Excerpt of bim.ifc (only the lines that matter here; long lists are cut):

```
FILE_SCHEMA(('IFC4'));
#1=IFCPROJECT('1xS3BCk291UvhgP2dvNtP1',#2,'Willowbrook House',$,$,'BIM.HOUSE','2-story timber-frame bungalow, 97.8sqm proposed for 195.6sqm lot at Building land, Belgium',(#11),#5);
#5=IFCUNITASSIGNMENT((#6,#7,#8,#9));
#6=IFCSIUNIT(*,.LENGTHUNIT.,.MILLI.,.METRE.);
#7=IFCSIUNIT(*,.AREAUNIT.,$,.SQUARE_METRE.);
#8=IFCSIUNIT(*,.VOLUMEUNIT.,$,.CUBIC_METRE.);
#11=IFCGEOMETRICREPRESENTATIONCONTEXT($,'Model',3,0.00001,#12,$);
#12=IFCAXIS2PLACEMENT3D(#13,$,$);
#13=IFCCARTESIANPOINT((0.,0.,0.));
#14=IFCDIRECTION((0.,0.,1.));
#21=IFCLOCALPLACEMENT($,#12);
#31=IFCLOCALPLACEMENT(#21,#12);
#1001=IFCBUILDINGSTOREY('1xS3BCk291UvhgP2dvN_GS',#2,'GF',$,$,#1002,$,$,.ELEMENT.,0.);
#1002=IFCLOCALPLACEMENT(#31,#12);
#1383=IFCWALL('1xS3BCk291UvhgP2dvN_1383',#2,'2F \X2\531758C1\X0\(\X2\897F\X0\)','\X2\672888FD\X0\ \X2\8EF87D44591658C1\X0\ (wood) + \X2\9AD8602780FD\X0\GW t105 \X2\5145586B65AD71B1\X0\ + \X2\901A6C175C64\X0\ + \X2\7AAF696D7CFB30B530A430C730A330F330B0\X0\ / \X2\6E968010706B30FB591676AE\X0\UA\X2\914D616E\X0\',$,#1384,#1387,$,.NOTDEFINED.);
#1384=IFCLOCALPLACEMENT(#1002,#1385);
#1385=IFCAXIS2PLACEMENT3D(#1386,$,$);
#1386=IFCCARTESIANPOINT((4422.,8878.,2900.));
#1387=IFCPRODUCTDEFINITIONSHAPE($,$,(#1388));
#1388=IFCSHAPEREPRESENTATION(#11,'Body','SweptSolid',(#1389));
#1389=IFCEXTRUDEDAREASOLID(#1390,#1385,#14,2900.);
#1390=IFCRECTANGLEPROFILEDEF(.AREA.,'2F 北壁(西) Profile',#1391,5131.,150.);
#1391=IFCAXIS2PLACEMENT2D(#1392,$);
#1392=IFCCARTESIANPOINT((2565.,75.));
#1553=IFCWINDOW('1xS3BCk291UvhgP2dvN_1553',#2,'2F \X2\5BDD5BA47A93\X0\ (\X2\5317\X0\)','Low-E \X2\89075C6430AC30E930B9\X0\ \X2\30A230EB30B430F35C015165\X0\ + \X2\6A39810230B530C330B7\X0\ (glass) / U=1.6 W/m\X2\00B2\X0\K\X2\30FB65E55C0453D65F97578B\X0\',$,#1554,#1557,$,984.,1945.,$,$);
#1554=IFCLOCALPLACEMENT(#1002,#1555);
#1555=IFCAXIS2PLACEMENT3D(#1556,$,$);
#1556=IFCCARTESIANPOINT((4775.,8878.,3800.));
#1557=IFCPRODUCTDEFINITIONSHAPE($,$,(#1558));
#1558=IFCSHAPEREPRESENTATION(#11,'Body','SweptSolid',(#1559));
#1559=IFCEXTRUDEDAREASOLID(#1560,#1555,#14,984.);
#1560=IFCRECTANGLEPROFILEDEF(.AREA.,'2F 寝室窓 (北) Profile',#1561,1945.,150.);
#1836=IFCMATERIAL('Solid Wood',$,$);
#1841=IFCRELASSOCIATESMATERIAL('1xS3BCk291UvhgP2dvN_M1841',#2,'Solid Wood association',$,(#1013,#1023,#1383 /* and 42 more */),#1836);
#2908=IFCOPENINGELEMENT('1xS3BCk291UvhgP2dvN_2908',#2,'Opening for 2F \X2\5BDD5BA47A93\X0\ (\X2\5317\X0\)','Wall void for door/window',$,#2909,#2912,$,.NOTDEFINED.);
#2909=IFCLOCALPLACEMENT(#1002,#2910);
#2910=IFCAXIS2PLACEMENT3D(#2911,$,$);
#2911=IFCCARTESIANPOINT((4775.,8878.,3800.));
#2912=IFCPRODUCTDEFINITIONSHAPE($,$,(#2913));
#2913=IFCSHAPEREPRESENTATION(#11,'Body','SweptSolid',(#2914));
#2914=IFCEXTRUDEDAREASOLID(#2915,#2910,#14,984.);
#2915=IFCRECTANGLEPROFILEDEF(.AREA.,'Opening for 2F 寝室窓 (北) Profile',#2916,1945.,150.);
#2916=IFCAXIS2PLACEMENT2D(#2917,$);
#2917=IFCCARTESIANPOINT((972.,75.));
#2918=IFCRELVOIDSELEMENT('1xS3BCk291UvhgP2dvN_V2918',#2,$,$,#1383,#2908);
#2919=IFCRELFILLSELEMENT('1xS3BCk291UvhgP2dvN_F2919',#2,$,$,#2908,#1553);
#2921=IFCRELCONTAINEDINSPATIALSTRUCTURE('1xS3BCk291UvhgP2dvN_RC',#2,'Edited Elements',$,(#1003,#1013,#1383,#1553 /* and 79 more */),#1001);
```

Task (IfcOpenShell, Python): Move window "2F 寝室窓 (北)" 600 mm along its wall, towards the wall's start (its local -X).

```python
import ifcopenshell
import ifcopenshell.api.geometry
import ifcopenshell.util.placement
import ifcopenshell.util.unit

model = ifcopenshell.open("bim.ifc")
unit_scale = ifcopenshell.util.unit.calculate_unit_scale(model)

window = model.by_id(1553)
opening = window.FillsVoids[0].RelatingOpeningElement
wall = opening.VoidsElements[0].RelatingBuildingElement

wall_matrix = ifcopenshell.util.placement.get_local_placement(wall.ObjectPlacement)
shift = wall_matrix[:3, 0] * -0.6 / unit_scale
before = ifcopenshell.util.placement.get_local_placement(window.ObjectPlacement)[:3, 3].copy()

# The window is not placed relative to its opening, so move both.
for product in (opening, window):
    matrix = ifcopenshell.util.placement.get_local_placement(product.ObjectPlacement)
    matrix[:3, 3] += shift
    ifcopenshell.api.geometry.edit_object_placement(model, product=product, matrix=matrix, is_si=False)

after = ifcopenshell.util.placement.get_local_placement(window.ObjectPlacement)[:3, 3]
print("window moved by", (after - before).round(3) + 0.0)

model.write("bim_updated.ifc")
```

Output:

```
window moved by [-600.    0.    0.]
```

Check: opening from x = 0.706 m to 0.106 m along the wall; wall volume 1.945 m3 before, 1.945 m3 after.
